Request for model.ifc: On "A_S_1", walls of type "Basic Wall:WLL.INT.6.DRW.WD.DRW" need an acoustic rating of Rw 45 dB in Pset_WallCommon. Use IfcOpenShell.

First a look at what the model holds.

```python
import ifcopenshell
import ifcopenshell.util.element

model = ifcopenshell.open("model.ifc")
print(model.schema)
storey = next(s for s in model.by_type("IfcBuildingStorey") if s.Name == "A_S_1")
walls = [e for e in ifcopenshell.util.element.get_decomposition(storey) if e.is_a("IfcWall")]
seen = {}
for e in walls:
    element_type = ifcopenshell.util.element.get_type(e)
    key = (element_type.Name if element_type != e and element_type else None, ifcopenshell.util.element.get_pset(e, "Pset_WallCommon", "AcousticRating"))
    seen[key] = seen.get(key, 0) + 1
for (name, value), count in sorted(seen.items(), key=str):
    print(count, "x", name, "|", value)
```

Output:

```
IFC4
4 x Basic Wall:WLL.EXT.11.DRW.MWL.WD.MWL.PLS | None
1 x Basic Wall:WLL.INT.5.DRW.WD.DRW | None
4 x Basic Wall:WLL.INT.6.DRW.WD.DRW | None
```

```python
import ifcopenshell
import ifcopenshell.api.pset
import ifcopenshell.util.element

model = ifcopenshell.open("model.ifc")

storey = next(s for s in model.by_type("IfcBuildingStorey") if s.Name == "A_S_1")
walls = [e for e in ifcopenshell.util.element.get_decomposition(storey) if e.is_a("IfcWall")]

count = 0
for e in walls:
    element_type = ifcopenshell.util.element.get_type(e)
    if element_type in (None, e) or element_type.Name != "Basic Wall:WLL.INT.6.DRW.WD.DRW":
        continue
    # add_pset returns the element's existing set when there is one.
    pset = ifcopenshell.api.pset.add_pset(model, product=e, name="Pset_WallCommon")
    ifcopenshell.api.pset.edit_pset(model, pset=pset, properties={"AcousticRating": "Rw 45 dB"})
    count += 1

print(count, "walls updated")

model.write("model_v2.ifc")
```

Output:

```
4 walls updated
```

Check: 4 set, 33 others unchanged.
